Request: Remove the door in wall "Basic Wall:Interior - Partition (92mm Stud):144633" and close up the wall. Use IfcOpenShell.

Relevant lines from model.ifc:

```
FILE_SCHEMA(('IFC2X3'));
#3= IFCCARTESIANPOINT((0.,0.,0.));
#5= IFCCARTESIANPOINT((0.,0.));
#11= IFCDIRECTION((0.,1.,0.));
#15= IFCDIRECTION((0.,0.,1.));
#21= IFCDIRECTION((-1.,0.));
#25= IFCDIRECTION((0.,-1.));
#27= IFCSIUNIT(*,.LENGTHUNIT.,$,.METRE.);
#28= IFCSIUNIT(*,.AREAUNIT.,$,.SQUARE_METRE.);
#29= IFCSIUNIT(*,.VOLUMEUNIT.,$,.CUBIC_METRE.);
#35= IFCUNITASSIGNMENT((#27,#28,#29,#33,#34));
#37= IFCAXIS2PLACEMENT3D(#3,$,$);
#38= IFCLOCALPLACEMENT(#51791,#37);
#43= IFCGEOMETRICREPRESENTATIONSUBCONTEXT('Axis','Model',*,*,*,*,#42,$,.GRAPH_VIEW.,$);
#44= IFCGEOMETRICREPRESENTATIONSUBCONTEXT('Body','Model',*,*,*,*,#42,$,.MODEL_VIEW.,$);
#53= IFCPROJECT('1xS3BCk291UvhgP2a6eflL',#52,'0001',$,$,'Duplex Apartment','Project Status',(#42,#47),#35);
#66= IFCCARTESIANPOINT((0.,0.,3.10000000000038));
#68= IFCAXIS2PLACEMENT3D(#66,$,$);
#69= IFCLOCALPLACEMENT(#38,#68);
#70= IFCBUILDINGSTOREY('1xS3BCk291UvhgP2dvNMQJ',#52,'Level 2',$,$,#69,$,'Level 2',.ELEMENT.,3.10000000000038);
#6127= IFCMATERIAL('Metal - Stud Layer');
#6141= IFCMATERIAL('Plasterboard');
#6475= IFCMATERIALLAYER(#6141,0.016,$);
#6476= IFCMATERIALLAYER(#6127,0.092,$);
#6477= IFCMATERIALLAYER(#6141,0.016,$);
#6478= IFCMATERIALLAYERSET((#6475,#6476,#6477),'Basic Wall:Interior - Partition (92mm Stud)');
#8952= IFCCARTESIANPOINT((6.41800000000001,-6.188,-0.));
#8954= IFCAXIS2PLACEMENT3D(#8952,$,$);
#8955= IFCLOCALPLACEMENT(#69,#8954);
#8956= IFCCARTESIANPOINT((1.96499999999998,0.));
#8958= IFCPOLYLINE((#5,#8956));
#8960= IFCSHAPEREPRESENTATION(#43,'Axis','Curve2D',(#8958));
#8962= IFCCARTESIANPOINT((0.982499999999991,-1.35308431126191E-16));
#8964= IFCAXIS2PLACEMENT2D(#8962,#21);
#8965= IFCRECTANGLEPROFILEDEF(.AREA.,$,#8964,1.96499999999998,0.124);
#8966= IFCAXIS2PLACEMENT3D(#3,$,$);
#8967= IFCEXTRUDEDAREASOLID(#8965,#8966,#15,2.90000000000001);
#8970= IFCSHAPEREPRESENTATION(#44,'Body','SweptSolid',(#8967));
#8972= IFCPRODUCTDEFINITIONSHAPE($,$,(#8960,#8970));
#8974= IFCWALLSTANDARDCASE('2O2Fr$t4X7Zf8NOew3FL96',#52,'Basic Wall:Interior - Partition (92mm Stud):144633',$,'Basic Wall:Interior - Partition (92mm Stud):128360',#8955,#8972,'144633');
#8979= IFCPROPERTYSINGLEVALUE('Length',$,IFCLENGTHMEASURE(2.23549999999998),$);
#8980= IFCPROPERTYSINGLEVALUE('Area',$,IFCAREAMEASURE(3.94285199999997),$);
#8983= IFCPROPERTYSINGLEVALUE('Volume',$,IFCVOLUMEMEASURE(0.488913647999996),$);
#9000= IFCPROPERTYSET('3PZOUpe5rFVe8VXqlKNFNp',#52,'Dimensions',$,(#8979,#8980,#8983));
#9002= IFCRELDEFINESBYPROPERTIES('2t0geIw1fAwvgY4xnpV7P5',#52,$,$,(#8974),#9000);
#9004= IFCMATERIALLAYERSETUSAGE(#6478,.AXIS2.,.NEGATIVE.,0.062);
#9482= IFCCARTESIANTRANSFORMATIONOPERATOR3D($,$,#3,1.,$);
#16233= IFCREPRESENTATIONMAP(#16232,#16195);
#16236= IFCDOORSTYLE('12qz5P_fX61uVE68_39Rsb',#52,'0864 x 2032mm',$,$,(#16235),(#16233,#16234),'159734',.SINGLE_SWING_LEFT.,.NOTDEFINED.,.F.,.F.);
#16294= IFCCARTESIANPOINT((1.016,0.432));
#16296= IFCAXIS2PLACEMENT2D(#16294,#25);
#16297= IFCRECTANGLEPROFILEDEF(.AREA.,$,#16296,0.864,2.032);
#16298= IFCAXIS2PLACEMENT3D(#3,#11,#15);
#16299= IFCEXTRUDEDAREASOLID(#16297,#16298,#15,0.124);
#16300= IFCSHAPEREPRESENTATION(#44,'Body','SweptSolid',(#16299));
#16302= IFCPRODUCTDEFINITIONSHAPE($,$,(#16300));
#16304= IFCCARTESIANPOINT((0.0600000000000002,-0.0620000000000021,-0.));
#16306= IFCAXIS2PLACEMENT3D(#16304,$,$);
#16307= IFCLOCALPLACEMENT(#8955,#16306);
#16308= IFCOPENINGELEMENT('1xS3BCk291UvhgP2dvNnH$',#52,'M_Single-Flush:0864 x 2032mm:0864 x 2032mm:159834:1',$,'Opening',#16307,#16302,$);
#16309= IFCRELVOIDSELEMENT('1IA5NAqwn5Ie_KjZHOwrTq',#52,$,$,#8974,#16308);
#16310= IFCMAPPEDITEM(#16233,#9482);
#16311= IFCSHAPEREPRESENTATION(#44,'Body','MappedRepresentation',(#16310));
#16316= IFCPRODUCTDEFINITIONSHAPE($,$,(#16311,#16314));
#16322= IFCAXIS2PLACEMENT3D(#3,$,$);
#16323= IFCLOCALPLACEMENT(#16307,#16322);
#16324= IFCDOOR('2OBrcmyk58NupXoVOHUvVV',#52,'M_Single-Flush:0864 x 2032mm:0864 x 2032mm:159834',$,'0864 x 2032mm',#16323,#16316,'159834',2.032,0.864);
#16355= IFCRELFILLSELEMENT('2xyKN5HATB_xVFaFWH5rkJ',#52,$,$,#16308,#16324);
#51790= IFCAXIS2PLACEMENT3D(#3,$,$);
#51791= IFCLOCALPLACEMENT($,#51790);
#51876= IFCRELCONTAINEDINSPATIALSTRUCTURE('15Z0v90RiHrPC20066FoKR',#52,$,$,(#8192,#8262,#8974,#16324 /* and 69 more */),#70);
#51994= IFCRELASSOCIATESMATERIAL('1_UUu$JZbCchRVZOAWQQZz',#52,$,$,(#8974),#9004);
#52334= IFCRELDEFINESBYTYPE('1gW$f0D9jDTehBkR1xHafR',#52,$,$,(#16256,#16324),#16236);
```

```python
import ifcopenshell
import ifcopenshell.api.feature
import ifcopenshell.api.pset
import ifcopenshell.api.root
import ifcopenshell.geom
import ifcopenshell.util.element
import ifcopenshell.util.shape
import ifcopenshell.util.unit

model = ifcopenshell.open("model.ifc")
area_scale = ifcopenshell.util.unit.calculate_unit_scale(model, "AREAUNIT")
volume_scale = ifcopenshell.util.unit.calculate_unit_scale(model, "VOLUMEUNIT")
settings = ifcopenshell.geom.settings()


def volume(element):
    """Net volume in cubic metres, openings subtracted."""
    shape = ifcopenshell.geom.create_shape(settings, element)
    return ifcopenshell.util.shape.get_volume(shape.geometry)


door = model.by_guid("2OBrcmyk58NupXoVOHUvVV")
opening = door.FillsVoids[0].RelatingOpeningElement
wall = opening.VoidsElements[0].RelatingBuildingElement
before = volume(wall)

ifcopenshell.api.root.remove_product(model, product=door)
ifcopenshell.api.feature.remove_feature(model, feature=opening)

after = volume(wall)
thickness = 0.124  # wall thickness in metres

# Update the wall's stored quantities.
pset = model.by_id(ifcopenshell.util.element.get_pset(wall, "Dimensions", should_inherit=False)["id"])
ifcopenshell.api.pset.edit_pset(model, pset=pset, properties={
    "Area": model.create_entity("IfcAreaMeasure", after / thickness / area_scale),
    "Volume": model.create_entity("IfcVolumeMeasure", after / volume_scale),
})

print(f"wall volume {before:.3f} -> {after:.3f} m3")

model.write("model_v2.ifc")
```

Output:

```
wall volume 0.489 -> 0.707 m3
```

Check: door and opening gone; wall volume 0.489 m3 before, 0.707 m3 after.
